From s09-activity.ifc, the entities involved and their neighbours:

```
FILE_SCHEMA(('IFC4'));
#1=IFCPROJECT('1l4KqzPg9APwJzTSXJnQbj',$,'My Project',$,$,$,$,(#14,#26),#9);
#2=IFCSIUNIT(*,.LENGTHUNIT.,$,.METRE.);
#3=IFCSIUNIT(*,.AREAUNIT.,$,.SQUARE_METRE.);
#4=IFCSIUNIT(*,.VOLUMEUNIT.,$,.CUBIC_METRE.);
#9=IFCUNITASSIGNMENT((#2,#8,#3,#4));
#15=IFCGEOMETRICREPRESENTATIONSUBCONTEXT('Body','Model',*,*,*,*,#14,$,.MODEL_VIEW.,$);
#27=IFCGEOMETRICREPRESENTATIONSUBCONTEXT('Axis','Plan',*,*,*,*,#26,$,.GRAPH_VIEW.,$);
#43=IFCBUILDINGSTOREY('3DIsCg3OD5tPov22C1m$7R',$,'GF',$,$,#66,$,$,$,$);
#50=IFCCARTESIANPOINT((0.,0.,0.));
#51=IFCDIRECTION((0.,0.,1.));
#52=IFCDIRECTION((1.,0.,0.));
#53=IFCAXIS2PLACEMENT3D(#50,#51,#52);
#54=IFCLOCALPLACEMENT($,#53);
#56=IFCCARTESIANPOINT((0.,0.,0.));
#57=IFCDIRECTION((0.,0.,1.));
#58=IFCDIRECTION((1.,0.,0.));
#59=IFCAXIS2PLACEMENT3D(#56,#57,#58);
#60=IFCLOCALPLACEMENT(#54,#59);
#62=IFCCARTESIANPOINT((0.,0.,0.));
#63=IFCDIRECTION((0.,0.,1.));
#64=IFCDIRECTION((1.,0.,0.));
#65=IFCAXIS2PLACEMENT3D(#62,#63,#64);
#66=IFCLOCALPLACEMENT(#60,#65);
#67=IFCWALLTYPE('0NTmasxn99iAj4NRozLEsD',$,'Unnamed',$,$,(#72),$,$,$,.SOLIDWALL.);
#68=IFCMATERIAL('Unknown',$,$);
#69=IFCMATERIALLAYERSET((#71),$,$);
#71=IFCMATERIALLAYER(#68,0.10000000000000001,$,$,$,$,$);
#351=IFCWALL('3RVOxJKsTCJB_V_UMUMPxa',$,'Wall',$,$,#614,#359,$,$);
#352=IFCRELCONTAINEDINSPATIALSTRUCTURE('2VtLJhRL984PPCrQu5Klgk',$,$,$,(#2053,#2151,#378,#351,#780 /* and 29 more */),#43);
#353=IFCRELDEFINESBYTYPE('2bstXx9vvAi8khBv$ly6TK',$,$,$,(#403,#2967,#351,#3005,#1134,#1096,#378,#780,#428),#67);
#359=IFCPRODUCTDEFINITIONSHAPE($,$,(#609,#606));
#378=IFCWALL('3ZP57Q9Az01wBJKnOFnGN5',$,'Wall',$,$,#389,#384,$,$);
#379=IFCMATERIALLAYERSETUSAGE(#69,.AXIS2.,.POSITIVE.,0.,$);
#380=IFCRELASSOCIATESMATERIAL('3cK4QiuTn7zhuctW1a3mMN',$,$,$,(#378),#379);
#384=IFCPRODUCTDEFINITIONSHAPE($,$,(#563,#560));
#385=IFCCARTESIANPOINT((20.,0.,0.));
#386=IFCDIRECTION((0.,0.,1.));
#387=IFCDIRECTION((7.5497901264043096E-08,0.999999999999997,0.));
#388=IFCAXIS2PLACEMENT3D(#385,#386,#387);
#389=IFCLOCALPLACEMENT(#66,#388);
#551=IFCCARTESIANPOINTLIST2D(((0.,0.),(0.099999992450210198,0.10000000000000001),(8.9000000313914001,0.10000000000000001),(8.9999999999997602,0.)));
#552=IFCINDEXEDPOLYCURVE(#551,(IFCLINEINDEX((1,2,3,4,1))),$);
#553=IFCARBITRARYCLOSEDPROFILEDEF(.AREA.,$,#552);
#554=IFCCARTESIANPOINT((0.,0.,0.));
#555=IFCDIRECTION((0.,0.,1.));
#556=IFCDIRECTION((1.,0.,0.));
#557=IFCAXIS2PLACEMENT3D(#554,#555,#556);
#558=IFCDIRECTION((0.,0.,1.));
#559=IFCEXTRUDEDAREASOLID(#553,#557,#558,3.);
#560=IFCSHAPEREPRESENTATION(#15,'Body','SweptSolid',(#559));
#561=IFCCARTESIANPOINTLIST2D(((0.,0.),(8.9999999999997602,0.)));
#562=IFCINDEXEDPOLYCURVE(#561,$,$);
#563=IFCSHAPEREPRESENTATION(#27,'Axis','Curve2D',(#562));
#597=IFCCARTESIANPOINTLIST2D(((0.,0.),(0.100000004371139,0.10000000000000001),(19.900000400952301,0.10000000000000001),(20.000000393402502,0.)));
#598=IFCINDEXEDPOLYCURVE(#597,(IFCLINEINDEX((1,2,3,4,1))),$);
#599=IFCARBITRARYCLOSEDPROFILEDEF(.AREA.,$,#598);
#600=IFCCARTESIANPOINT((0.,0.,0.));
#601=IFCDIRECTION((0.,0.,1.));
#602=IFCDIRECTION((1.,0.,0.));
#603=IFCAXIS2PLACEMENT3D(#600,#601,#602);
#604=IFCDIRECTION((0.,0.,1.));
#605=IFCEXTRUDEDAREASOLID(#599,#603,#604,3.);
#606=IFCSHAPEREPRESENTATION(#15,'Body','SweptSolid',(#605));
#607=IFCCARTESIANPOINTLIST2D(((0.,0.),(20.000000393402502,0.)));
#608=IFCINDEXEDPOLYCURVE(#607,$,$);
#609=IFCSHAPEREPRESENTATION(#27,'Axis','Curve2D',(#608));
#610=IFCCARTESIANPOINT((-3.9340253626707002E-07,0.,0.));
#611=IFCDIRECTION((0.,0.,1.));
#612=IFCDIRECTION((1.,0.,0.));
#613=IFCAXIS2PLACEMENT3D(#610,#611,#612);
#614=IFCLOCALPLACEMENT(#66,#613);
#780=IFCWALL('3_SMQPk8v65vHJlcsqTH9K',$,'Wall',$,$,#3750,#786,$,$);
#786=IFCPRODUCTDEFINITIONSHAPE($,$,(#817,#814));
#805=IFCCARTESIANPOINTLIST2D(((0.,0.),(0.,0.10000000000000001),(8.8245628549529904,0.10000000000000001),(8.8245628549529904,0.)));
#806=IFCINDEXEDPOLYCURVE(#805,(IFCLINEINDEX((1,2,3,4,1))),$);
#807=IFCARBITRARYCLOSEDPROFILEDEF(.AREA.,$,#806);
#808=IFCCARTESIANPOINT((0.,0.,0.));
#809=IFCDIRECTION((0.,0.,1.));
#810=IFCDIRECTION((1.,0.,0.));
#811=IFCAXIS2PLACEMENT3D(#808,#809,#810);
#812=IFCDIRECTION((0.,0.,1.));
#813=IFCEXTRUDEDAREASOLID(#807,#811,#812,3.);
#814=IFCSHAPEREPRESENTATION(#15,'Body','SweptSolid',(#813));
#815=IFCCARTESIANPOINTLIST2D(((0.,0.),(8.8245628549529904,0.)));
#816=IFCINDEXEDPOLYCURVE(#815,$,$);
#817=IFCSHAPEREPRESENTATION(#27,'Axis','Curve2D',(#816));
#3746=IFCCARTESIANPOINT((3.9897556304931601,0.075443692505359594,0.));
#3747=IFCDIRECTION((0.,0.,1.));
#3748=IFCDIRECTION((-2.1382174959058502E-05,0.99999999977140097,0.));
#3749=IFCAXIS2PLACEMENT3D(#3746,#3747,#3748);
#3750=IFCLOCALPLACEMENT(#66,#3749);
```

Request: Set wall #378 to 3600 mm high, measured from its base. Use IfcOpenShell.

```python
import ifcopenshell
import ifcopenshell.geom
import ifcopenshell.util.representation
import ifcopenshell.util.shape

model = ifcopenshell.open("s09-activity.ifc")
settings = ifcopenshell.geom.settings()


def volume(element):
    """Net volume in cubic metres, openings subtracted."""
    shape = ifcopenshell.geom.create_shape(settings, element)
    return ifcopenshell.util.shape.get_volume(shape.geometry)


wall = model.by_guid("3ZP57Q9Az01wBJKnOFnGN5")
before = volume(wall)

body = ifcopenshell.util.representation.get_representation(wall, "Model", "Body")
solid = body.Items[0]
old_height = solid.Depth
solid.Depth = 3.6
after = volume(wall)

print(f"height {old_height:g} -> {solid.Depth:g}, volume {before:.3f} -> {after:.3f} m3")

model.write("s09-activity_edited.ifc")
```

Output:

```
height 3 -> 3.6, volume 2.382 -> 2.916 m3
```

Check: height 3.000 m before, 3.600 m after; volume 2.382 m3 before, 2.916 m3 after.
